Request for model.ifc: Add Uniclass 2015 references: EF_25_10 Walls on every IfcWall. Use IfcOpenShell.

First a look at what the model holds.

```python
import ifcopenshell

model = ifcopenshell.open("model.ifc")
print(model.schema)
print("classifications:", [c.Name for c in model.by_type("IfcClassification")])
for ifc_class in ("IfcDoor", "IfcRoof", "IfcStair", "IfcWall", "IfcWindow"):
    print(ifc_class, len(model.by_type(ifc_class)))
```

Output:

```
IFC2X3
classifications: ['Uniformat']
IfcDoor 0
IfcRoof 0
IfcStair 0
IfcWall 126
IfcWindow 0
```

```python
import ifcopenshell
import ifcopenshell.api.classification

model = ifcopenshell.open("model.ifc")

# IFC2X3 requires Source and Edition and has no link from the project to the system.
system = model.create_entity("IfcClassification", Source="NBS", Edition="2015", Name="Uniclass 2015")

codes = {
    "IfcWall": ("EF_25_10", "Walls"),
}
for ifc_class, (code, name) in codes.items():
    products = model.by_type(ifc_class)
    ifcopenshell.api.classification.add_reference(
        model, products=products, classification=system, identification=code, name=name
    )
    print(code, len(products))

model.write("model_edited.ifc")
```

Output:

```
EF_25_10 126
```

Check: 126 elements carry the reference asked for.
